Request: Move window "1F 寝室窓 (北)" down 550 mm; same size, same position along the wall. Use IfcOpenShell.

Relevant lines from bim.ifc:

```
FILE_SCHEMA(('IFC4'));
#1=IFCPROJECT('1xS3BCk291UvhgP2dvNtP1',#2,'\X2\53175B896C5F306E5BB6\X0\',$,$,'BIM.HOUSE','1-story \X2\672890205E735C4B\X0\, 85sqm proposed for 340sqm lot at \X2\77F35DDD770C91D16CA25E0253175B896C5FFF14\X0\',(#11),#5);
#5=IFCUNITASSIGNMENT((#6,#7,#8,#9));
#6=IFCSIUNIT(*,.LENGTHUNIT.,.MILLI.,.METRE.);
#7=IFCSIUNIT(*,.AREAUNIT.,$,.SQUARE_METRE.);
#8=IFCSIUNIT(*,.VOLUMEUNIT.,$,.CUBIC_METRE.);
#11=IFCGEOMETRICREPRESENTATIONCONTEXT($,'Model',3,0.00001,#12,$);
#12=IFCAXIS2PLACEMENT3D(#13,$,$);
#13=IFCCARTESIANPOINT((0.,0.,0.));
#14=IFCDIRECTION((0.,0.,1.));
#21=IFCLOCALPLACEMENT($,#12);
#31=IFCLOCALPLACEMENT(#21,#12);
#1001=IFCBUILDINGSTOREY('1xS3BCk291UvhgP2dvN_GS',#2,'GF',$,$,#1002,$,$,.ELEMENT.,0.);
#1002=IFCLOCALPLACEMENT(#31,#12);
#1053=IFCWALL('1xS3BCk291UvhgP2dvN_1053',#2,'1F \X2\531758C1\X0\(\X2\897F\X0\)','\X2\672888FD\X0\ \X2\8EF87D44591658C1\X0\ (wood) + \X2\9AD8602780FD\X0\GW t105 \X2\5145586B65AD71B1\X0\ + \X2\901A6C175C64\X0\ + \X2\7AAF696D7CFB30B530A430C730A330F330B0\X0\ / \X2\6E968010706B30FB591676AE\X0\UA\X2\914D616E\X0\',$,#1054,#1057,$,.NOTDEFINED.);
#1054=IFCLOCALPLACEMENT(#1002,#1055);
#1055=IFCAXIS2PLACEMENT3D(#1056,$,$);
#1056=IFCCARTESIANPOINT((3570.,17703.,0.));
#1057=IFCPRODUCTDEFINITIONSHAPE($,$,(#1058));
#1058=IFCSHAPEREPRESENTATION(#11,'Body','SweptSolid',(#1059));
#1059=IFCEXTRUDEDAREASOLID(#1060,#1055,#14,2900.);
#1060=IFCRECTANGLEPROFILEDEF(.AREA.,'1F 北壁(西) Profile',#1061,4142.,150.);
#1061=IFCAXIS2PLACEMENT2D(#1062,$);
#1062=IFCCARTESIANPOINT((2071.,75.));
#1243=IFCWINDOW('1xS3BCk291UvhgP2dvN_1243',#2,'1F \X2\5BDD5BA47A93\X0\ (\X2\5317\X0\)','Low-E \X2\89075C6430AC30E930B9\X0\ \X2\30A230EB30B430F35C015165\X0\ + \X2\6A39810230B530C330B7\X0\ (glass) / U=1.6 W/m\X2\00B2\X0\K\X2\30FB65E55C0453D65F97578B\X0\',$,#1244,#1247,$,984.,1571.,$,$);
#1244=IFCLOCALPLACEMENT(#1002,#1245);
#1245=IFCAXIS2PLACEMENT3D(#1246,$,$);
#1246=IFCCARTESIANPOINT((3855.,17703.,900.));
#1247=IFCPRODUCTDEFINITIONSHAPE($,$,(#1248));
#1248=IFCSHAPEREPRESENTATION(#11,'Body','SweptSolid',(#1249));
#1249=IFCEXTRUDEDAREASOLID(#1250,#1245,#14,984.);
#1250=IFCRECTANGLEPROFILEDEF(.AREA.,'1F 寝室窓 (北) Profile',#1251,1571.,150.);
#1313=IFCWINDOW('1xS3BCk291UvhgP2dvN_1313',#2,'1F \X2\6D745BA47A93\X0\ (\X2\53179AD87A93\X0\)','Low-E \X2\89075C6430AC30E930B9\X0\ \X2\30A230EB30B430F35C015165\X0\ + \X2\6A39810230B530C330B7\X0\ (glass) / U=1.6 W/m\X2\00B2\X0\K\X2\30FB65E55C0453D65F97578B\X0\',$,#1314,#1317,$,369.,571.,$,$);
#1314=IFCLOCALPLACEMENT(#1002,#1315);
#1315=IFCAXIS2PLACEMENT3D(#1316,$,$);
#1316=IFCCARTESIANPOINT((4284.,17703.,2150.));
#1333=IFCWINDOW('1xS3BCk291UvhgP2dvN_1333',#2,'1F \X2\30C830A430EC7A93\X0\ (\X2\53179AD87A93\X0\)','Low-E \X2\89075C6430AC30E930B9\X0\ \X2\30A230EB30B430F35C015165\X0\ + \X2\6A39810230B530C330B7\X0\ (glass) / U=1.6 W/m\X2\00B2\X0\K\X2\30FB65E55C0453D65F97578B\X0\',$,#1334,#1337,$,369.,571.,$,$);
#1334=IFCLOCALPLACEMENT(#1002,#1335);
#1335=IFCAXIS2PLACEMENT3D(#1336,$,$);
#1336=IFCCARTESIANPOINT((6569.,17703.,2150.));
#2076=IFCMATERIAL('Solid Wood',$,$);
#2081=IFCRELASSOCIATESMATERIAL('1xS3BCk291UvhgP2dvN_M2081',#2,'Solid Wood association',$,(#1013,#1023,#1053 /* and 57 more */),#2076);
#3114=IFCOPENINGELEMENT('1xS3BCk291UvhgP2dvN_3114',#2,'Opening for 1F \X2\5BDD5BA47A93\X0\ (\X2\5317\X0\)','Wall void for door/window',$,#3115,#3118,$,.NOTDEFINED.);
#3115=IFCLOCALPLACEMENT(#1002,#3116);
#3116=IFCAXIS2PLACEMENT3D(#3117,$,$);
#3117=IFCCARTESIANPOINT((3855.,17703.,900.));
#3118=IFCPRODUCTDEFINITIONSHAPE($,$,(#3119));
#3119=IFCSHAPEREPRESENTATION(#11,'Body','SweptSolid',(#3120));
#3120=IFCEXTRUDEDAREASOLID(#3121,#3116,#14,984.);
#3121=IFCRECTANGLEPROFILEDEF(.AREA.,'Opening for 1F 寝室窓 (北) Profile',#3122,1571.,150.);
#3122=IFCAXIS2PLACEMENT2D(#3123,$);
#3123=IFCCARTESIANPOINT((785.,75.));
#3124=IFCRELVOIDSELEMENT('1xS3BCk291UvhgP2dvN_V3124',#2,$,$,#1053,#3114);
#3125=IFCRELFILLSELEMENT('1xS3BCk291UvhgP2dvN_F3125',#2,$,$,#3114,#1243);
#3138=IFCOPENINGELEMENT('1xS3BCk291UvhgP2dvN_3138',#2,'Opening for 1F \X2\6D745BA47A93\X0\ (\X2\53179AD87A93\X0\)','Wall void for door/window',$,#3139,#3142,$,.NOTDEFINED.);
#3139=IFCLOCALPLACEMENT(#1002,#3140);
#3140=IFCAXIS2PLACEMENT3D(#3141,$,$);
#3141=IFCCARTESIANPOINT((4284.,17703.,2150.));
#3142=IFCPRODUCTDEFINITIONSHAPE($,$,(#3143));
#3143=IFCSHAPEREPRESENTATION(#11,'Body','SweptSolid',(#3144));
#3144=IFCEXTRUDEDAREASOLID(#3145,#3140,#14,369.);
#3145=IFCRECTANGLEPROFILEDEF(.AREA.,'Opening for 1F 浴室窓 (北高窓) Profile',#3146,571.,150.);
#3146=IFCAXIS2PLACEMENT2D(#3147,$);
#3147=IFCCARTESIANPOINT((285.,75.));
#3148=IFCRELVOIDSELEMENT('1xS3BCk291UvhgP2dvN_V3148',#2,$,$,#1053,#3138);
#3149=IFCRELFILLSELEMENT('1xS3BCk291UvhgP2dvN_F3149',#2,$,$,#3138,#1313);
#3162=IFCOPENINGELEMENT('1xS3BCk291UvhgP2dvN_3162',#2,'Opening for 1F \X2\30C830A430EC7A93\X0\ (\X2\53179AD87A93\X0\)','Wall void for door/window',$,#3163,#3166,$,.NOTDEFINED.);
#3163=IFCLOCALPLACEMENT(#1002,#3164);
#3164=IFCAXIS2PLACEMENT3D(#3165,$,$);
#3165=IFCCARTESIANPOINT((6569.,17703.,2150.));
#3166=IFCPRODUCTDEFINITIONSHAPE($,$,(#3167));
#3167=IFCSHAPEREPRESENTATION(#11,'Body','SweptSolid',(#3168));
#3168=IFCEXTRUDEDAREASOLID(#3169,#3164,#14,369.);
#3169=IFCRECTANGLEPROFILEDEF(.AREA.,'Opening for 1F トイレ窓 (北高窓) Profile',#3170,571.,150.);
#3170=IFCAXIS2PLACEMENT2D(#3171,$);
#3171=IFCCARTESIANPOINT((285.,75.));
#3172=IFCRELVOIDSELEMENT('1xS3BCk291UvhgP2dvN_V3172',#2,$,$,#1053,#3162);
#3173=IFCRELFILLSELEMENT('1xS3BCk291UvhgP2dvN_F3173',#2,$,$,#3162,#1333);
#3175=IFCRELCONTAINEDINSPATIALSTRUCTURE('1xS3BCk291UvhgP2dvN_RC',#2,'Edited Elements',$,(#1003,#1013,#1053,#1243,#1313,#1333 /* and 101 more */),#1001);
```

```python
import numpy as np
import ifcopenshell
import ifcopenshell.api.geometry
import ifcopenshell.util.placement
import ifcopenshell.util.unit

model = ifcopenshell.open("bim.ifc")
unit_scale = ifcopenshell.util.unit.calculate_unit_scale(model)

window = model.by_id(1243)
opening = window.FillsVoids[0].RelatingOpeningElement
dz = -550.0

shift = np.array([0.0, 0.0, dz])
# The window is not placed relative to its opening, so move both.
for product in (opening, window):
    matrix = ifcopenshell.util.placement.get_local_placement(product.ObjectPlacement)
    matrix[:3, 3] += shift
    ifcopenshell.api.geometry.edit_object_placement(model, product=product, matrix=matrix, is_si=False)

print(f"moved by {dz * unit_scale:+.3f} m")

model.write("bim_updated.ifc")
```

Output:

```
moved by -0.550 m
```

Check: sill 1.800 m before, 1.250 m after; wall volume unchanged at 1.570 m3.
